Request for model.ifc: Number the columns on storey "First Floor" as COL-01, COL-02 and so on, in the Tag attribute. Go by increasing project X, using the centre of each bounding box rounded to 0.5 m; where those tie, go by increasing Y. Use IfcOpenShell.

First a look at what the model holds.

```python
import ifcopenshell
import ifcopenshell.util.element
import ifcopenshell.util.placement

model = ifcopenshell.open("model.ifc")
print(model.schema)
storey = next(s for s in model.by_type("IfcBuildingStorey") if s.Name == "First Floor")
columns = [e for e in ifcopenshell.util.element.get_decomposition(storey) if e.is_a("IfcColumn")]
for e in sorted(columns, key=lambda e: e.id()):
    origin = ifcopenshell.util.placement.get_local_placement(e.ObjectPlacement)[:3, 3]
    print(e.id(), e.Tag, e.Name, origin.round(2) + 0.0, sep=" | ")
```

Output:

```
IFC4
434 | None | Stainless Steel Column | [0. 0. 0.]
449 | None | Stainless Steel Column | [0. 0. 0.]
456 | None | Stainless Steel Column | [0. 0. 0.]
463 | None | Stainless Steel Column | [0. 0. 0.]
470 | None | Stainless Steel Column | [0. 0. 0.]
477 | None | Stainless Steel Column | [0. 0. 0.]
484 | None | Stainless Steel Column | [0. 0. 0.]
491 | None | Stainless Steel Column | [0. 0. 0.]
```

```python
import ifcopenshell
import ifcopenshell.geom
import ifcopenshell.util.element
import ifcopenshell.util.shape

model = ifcopenshell.open("model.ifc")
settings = ifcopenshell.geom.settings()
settings.set("use-world-coords", True)


def centre(element):
    shape = ifcopenshell.geom.create_shape(settings, element)
    return ifcopenshell.util.shape.get_bbox_centroid(shape.geometry)


storey = next(s for s in model.by_type("IfcBuildingStorey") if s.Name == "First Floor")
columns = [e for e in ifcopenshell.util.element.get_decomposition(storey) if e.is_a("IfcColumn")]

# Insertion points can sit at a corner or the storey origin, so sort by the geometry (in metres).
centres = {e: centre(e) for e in columns}
columns.sort(key=lambda e: (round(centres[e][0] / 0.5), centres[e][1]))

for i, e in enumerate(columns, start=1):
    number = f"COL-{i:02d}"
    e.Tag = number
    print(e.id(), number)

model.write("model_rev.ifc")
```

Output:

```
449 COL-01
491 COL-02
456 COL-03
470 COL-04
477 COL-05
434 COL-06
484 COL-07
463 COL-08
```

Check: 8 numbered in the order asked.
